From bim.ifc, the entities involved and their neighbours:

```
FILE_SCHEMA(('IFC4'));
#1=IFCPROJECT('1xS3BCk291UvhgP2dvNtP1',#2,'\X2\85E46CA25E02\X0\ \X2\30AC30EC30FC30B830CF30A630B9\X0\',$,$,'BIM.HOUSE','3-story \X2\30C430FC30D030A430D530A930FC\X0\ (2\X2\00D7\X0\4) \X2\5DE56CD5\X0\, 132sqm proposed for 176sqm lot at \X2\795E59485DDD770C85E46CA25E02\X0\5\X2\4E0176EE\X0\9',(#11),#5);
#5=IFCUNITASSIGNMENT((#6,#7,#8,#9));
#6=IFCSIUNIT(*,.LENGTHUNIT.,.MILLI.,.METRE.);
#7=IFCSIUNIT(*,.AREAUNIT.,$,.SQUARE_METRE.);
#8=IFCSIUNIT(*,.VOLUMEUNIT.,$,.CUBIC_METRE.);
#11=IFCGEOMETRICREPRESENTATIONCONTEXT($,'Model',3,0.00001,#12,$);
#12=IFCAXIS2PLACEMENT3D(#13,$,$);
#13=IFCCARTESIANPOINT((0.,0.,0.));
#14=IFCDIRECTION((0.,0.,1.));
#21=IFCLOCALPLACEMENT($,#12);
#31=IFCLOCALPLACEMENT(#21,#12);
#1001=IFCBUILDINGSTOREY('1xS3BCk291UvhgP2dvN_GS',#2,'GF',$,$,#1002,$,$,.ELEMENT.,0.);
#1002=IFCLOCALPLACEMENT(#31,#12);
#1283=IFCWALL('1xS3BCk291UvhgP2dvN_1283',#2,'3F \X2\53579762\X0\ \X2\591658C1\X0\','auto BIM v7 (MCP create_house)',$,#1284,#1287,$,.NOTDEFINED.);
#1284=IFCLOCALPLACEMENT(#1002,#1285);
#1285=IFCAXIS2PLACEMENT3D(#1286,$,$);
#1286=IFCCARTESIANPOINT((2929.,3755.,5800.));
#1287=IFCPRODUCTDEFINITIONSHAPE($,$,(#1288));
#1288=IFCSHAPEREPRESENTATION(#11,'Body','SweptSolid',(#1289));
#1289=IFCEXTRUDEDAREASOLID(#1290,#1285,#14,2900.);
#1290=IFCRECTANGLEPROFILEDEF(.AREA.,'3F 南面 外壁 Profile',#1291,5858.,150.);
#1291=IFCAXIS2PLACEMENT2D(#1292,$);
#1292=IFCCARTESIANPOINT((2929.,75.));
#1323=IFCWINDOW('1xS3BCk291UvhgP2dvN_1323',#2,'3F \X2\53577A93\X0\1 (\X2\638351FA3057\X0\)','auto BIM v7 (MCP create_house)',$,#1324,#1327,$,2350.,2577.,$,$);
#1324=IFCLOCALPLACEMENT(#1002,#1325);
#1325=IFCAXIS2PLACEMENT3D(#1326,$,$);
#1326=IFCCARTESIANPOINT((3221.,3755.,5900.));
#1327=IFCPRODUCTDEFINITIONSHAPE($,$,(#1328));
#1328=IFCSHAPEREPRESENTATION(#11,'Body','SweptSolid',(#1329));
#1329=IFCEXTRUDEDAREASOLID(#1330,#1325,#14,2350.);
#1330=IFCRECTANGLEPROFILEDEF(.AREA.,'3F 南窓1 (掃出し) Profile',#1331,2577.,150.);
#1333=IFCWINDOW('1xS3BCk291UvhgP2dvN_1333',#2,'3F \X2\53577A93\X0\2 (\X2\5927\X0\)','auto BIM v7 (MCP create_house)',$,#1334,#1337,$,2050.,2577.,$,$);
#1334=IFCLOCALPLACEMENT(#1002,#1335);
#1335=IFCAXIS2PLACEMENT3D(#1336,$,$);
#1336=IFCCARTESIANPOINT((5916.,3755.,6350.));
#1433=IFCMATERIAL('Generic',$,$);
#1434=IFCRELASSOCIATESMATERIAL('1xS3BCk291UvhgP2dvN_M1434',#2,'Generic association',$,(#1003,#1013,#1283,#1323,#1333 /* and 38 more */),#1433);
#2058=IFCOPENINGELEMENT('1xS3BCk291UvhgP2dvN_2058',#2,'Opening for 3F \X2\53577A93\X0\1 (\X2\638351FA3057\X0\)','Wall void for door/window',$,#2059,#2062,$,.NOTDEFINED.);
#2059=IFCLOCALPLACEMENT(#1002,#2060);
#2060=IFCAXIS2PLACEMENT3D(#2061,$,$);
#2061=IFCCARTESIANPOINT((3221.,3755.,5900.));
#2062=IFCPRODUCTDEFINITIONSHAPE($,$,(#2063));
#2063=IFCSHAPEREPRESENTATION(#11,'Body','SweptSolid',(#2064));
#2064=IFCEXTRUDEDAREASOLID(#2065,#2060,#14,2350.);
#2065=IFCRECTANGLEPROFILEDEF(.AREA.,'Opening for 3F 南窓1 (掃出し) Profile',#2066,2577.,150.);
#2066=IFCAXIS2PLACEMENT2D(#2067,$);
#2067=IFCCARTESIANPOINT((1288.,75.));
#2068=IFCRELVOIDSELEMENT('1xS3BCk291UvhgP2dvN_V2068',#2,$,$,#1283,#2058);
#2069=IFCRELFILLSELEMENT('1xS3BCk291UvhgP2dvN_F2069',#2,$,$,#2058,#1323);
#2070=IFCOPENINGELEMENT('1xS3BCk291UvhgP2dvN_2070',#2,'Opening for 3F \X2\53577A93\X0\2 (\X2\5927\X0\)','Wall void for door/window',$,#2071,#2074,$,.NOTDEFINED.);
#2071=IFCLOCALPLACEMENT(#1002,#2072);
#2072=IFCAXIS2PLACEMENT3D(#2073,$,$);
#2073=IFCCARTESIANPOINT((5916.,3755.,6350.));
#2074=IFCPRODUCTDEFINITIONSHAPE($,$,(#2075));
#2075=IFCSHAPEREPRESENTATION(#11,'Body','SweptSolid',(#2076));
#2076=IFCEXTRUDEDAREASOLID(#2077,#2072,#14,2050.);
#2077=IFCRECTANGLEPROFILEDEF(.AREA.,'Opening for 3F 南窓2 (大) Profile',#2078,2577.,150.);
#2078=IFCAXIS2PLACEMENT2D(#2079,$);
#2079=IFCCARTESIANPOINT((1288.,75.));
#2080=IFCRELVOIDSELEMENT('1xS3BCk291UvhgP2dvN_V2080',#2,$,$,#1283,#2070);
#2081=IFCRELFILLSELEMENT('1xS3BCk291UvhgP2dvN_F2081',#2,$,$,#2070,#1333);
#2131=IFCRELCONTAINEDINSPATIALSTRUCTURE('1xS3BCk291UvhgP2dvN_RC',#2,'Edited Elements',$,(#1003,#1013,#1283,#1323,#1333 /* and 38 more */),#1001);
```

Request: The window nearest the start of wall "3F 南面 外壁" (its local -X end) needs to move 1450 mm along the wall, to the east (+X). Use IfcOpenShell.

```python
import ifcopenshell
import ifcopenshell.api.geometry
import ifcopenshell.util.placement

model = ifcopenshell.open("bim.ifc")

window = model.by_guid("1xS3BCk291UvhgP2dvN_1323")
opening = window.FillsVoids[0].RelatingOpeningElement
wall = opening.VoidsElements[0].RelatingBuildingElement

wall_matrix = ifcopenshell.util.placement.get_local_placement(wall.ObjectPlacement)
shift = wall_matrix[:3, 0] * 1450.0
before = ifcopenshell.util.placement.get_local_placement(window.ObjectPlacement)[:3, 3].copy()

# The window is not placed relative to its opening, so move both.
for product in (opening, window):
    matrix = ifcopenshell.util.placement.get_local_placement(product.ObjectPlacement)
    matrix[:3, 3] += shift
    ifcopenshell.api.geometry.edit_object_placement(model, product=product, matrix=matrix, is_si=False)

after = ifcopenshell.util.placement.get_local_placement(window.ObjectPlacement)[:3, 3]
print("window moved by", (after - before).round(3) + 0.0)

model.write("bim_rev.ifc")
```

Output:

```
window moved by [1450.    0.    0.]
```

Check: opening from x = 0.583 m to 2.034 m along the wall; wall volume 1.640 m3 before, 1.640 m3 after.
